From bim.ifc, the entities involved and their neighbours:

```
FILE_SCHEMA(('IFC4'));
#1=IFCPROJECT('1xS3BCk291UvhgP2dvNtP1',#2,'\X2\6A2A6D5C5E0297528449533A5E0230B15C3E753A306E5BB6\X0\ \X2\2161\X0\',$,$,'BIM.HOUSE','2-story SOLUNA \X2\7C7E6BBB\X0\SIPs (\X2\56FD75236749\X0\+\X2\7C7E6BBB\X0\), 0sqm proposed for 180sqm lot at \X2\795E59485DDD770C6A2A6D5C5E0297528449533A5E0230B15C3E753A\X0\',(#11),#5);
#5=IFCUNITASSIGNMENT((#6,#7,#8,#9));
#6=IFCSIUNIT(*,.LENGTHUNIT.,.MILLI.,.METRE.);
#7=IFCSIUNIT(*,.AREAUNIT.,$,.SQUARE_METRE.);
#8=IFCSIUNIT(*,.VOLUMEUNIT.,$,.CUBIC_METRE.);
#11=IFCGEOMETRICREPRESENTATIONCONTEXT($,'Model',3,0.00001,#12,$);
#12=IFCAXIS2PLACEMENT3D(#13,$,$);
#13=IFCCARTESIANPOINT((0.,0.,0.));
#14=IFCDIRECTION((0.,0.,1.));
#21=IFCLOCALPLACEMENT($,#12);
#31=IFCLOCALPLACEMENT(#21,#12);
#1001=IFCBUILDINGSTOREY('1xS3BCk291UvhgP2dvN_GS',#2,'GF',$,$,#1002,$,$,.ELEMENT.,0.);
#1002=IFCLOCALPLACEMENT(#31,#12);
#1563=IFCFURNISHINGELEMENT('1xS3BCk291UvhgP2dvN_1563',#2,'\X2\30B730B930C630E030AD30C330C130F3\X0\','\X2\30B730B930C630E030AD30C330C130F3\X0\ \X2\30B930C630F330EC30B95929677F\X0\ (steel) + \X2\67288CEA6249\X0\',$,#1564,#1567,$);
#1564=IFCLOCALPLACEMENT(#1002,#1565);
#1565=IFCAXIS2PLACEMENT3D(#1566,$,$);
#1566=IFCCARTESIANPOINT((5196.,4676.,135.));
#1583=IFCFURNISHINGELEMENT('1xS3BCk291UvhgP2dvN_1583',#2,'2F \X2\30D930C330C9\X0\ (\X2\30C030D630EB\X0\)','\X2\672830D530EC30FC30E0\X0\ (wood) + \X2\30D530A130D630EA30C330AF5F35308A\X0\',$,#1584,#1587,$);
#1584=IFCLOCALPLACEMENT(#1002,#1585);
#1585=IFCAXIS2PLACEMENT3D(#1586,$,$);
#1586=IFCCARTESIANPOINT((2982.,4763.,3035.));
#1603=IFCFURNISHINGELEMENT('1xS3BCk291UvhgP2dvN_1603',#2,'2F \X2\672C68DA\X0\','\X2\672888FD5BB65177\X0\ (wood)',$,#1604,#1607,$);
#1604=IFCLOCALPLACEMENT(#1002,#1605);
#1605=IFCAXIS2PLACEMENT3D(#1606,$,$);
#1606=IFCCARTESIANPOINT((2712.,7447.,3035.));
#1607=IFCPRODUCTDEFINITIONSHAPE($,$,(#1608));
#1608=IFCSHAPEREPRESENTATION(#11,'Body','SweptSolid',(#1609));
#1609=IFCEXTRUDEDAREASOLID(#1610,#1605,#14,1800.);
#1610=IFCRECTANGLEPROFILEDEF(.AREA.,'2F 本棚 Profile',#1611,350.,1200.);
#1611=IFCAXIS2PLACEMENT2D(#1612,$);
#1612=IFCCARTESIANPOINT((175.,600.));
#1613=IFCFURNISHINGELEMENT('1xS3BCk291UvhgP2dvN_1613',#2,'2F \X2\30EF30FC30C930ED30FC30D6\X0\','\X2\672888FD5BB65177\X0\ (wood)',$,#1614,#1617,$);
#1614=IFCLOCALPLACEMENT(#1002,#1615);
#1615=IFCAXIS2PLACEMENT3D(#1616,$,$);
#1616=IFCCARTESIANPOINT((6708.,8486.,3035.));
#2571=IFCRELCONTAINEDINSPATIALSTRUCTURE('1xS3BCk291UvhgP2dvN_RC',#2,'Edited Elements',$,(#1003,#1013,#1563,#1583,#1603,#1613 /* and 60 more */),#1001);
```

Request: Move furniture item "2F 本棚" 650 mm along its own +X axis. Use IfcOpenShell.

```python
import ifcopenshell
import ifcopenshell.api.geometry
import ifcopenshell.util.placement

model = ifcopenshell.open("bim.ifc")

item = model.by_id(1603)
matrix = ifcopenshell.util.placement.get_local_placement(item.ObjectPlacement)
matrix[:3, 3] += matrix[:3, 0] * 650.0
ifcopenshell.api.geometry.edit_object_placement(model, product=item, matrix=matrix, is_si=False)

print(ifcopenshell.util.placement.get_local_placement(item.ObjectPlacement).round(3) + 0.0)

model.write("bim_rev.ifc")
```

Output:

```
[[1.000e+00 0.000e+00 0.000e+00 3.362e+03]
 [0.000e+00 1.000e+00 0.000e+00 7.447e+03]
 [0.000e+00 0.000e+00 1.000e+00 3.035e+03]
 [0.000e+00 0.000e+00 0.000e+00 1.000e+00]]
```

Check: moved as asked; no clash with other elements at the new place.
